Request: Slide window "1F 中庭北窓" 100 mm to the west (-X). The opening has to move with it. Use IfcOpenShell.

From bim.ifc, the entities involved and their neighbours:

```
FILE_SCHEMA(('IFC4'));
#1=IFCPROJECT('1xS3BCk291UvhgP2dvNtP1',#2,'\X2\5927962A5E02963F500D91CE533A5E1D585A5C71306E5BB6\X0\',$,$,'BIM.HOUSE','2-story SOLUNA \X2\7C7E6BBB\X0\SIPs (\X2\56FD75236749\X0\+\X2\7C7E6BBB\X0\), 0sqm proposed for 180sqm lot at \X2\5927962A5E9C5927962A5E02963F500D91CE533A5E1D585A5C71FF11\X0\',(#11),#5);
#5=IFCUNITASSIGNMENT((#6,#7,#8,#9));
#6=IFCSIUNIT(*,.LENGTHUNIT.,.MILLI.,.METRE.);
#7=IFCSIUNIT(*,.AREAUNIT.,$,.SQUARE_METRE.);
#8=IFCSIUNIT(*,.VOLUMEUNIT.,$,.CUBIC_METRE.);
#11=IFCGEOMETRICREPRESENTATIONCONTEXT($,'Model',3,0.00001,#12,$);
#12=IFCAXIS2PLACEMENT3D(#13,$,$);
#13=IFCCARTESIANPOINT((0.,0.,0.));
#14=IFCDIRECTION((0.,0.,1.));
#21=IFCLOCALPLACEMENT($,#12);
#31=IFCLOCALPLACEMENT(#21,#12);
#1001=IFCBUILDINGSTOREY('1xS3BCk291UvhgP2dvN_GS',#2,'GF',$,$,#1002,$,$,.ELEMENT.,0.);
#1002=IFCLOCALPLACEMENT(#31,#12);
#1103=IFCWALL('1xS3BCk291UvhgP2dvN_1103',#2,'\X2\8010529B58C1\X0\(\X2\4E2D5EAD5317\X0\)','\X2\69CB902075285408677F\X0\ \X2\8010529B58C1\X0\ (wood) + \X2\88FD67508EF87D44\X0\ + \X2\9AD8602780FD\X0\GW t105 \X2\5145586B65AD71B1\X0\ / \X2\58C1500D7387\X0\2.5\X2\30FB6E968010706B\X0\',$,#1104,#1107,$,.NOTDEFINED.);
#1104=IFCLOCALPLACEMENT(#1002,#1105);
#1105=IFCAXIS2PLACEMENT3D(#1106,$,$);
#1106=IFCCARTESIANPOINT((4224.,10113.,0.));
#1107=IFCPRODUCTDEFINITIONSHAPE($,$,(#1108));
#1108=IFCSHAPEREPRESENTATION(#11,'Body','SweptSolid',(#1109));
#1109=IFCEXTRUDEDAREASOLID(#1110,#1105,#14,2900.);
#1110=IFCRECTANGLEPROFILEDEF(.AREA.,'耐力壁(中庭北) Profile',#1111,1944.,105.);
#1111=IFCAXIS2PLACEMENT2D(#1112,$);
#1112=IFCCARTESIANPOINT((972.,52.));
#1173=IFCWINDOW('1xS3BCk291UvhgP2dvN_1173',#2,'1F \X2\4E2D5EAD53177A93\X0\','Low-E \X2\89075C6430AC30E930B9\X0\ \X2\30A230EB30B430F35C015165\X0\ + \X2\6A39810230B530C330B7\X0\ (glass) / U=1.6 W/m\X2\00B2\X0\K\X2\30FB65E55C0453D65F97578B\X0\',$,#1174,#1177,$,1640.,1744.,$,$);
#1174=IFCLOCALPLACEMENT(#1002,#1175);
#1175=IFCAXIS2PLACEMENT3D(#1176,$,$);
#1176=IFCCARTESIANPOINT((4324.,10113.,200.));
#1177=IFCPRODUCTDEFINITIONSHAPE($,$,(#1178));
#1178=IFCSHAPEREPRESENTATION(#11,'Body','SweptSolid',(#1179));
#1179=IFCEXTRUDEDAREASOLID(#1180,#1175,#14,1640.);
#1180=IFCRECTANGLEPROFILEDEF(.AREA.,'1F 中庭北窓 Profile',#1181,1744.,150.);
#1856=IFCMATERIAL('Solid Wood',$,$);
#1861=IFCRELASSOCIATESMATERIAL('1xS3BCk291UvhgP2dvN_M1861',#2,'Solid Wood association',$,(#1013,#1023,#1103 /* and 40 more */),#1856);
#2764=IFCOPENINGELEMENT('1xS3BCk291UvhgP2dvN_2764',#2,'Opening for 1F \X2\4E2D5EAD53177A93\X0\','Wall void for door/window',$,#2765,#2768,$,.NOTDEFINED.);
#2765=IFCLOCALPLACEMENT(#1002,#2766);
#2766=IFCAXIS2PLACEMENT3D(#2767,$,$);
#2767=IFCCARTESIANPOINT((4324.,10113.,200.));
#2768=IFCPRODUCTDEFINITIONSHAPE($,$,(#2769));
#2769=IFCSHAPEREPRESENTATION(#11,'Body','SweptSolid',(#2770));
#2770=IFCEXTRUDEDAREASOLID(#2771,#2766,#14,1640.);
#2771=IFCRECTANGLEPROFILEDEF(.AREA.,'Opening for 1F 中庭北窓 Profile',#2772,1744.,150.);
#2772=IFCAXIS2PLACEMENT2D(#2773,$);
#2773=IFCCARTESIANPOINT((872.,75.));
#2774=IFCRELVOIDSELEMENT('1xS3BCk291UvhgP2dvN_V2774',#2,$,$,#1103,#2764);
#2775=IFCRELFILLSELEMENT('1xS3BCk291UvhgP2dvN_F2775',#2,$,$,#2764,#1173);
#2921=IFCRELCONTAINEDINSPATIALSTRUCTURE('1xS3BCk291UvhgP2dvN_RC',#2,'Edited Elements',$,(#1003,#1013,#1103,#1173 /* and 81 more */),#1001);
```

```python
import ifcopenshell
import ifcopenshell.api.geometry
import ifcopenshell.util.placement
import ifcopenshell.util.unit

model = ifcopenshell.open("bim.ifc")
unit_scale = ifcopenshell.util.unit.calculate_unit_scale(model)

window = model.by_id(1173)
opening = window.FillsVoids[0].RelatingOpeningElement
wall = opening.VoidsElements[0].RelatingBuildingElement

wall_matrix = ifcopenshell.util.placement.get_local_placement(wall.ObjectPlacement)
shift = wall_matrix[:3, 0] * -0.1 / unit_scale
before = ifcopenshell.util.placement.get_local_placement(window.ObjectPlacement)[:3, 3].copy()

# The window is not placed relative to its opening, so move both.
for product in (opening, window):
    matrix = ifcopenshell.util.placement.get_local_placement(product.ObjectPlacement)
    matrix[:3, 3] += shift
    ifcopenshell.api.geometry.edit_object_placement(model, product=product, matrix=matrix, is_si=False)

after = ifcopenshell.util.placement.get_local_placement(window.ObjectPlacement)[:3, 3]
print("window moved by", (after - before).round(3) + 0.0)

model.write("bim_edited.ifc")
```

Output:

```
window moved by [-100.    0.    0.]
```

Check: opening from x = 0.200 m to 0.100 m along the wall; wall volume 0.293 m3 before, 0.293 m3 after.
